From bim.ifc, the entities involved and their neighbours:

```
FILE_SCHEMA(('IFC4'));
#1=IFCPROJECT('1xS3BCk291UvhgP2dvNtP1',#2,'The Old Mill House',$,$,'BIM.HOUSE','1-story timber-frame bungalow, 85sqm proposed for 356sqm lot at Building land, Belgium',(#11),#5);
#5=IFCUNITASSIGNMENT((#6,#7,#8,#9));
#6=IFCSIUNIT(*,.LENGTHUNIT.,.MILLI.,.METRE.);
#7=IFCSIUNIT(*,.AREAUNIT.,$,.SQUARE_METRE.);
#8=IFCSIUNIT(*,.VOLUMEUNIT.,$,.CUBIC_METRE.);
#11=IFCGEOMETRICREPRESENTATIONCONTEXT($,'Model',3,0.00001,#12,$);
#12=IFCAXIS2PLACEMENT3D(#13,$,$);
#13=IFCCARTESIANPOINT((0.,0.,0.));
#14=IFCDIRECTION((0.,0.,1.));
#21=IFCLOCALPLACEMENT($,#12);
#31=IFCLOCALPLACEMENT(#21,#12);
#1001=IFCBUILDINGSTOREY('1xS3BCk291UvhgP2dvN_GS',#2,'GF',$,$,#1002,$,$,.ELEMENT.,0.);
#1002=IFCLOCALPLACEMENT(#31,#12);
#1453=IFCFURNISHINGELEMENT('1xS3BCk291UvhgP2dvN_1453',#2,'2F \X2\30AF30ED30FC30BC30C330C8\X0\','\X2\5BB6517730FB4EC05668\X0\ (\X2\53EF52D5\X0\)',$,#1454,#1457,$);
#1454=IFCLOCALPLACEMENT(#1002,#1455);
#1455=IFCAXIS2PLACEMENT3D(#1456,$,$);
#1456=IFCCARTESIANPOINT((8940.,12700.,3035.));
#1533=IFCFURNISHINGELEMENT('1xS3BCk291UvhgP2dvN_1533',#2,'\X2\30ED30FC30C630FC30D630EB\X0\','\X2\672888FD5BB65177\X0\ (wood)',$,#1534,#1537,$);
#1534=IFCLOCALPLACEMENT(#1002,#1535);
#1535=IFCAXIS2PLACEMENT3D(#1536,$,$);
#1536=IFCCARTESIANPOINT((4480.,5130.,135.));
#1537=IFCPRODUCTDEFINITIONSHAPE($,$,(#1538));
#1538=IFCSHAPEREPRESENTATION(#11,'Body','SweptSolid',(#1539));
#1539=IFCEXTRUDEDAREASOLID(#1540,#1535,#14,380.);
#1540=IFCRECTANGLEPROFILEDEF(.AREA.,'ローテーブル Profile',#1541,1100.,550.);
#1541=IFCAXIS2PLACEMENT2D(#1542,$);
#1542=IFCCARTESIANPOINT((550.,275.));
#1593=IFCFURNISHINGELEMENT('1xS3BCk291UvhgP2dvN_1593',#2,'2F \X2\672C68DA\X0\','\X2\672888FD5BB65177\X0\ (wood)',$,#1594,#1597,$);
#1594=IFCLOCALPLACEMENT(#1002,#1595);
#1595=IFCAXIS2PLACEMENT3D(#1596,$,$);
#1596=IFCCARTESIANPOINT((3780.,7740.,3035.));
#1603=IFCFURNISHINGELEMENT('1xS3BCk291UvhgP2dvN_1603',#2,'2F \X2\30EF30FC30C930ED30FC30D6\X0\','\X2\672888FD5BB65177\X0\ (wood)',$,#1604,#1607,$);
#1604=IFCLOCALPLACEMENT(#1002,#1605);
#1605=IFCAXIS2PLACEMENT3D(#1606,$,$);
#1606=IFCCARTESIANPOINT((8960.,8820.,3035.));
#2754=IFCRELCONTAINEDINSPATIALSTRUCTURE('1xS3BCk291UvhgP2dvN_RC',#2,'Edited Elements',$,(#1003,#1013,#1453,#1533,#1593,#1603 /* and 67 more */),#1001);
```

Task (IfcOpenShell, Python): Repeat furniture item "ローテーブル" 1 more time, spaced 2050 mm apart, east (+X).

```python
import numpy as np
import ifcopenshell
import ifcopenshell.api.geometry
import ifcopenshell.api.root
import ifcopenshell.util.element
import ifcopenshell.util.placement
import ifcopenshell.util.unit

model = ifcopenshell.open("bim.ifc")
unit_scale = ifcopenshell.util.unit.calculate_unit_scale(model)


def reuse_history(source, copy):
    """copy_class also copies each property set's owner history, people and application; keep the originals."""
    for rel in copy.IsDefinedBy:
        if rel.is_a("IfcRelDefinesByProperties") and (history := rel.RelatingPropertyDefinition.OwnerHistory):
            rel.RelatingPropertyDefinition.OwnerHistory = source.OwnerHistory
            ifcopenshell.util.element.remove_deep2(model, history)


source = model.by_guid("1xS3BCk291UvhgP2dvN_1533")
base = ifcopenshell.util.placement.get_local_placement(source.ObjectPlacement)
step = np.array([1.0, 0.0, 0.0]) * 2.05 / unit_scale

for i in range(1, 2):
    copy = ifcopenshell.api.root.copy_class(model, product=source)
    copy.Representation = ifcopenshell.util.element.copy_deep(
        model, source.Representation, exclude=["IfcGeometricRepresentationContext", "IfcRepresentationMap"]
    )
    reuse_history(source, copy)
    matrix = base.copy()
    matrix[:3, 3] += i * step
    print("added at", matrix[:3, 3].round(3) + 0.0)
    ifcopenshell.api.geometry.edit_object_placement(model, product=copy, matrix=matrix, is_si=False)

model.write("bim_edited.ifc")
```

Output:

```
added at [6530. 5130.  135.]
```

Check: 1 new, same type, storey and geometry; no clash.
